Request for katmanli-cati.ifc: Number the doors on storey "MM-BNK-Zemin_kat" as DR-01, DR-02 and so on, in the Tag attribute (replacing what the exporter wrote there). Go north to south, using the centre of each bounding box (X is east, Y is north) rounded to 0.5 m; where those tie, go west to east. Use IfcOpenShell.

First a look at what the model holds.

```python
import ifcopenshell
import ifcopenshell.util.element
import ifcopenshell.util.placement

model = ifcopenshell.open("katmanli-cati.ifc")
print(model.schema)
storey = next(s for s in model.by_type("IfcBuildingStorey") if s.Name == "MM-BNK-Zemin_kat")
doors = [e for e in ifcopenshell.util.element.get_decomposition(storey) if e.is_a("IfcDoor")]
for e in sorted(doors, key=lambda e: e.id()):
    origin = ifcopenshell.util.placement.get_local_placement(e.ObjectPlacement)[:3, 3]
    print(e.id(), e.Tag, e.Name, origin.round(2) + 0.0, sep=" | ")
```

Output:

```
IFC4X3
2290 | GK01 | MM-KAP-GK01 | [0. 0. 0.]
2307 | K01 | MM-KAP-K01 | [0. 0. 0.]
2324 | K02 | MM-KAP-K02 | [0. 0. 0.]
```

```python
import ifcopenshell
import ifcopenshell.geom
import ifcopenshell.util.element
import ifcopenshell.util.shape

model = ifcopenshell.open("katmanli-cati.ifc")
settings = ifcopenshell.geom.settings()
settings.set("use-world-coords", True)


def centre(element):
    shape = ifcopenshell.geom.create_shape(settings, element)
    return ifcopenshell.util.shape.get_bbox_centroid(shape.geometry)


storey = next(s for s in model.by_type("IfcBuildingStorey") if s.Name == "MM-BNK-Zemin_kat")
doors = [e for e in ifcopenshell.util.element.get_decomposition(storey) if e.is_a("IfcDoor")]

# Insertion points can sit at a corner or the storey origin, so sort by the geometry (in metres).
centres = {e: centre(e) for e in doors}
doors.sort(key=lambda e: (-round(centres[e][1] / 0.5), centres[e][0]))

for i, e in enumerate(doors, start=1):
    number = f"DR-{i:02d}"
    e.Tag = number
    print(e.id(), number)

model.write("katmanli-cati_v2.ifc")
```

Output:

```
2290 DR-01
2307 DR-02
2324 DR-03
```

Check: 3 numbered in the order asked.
